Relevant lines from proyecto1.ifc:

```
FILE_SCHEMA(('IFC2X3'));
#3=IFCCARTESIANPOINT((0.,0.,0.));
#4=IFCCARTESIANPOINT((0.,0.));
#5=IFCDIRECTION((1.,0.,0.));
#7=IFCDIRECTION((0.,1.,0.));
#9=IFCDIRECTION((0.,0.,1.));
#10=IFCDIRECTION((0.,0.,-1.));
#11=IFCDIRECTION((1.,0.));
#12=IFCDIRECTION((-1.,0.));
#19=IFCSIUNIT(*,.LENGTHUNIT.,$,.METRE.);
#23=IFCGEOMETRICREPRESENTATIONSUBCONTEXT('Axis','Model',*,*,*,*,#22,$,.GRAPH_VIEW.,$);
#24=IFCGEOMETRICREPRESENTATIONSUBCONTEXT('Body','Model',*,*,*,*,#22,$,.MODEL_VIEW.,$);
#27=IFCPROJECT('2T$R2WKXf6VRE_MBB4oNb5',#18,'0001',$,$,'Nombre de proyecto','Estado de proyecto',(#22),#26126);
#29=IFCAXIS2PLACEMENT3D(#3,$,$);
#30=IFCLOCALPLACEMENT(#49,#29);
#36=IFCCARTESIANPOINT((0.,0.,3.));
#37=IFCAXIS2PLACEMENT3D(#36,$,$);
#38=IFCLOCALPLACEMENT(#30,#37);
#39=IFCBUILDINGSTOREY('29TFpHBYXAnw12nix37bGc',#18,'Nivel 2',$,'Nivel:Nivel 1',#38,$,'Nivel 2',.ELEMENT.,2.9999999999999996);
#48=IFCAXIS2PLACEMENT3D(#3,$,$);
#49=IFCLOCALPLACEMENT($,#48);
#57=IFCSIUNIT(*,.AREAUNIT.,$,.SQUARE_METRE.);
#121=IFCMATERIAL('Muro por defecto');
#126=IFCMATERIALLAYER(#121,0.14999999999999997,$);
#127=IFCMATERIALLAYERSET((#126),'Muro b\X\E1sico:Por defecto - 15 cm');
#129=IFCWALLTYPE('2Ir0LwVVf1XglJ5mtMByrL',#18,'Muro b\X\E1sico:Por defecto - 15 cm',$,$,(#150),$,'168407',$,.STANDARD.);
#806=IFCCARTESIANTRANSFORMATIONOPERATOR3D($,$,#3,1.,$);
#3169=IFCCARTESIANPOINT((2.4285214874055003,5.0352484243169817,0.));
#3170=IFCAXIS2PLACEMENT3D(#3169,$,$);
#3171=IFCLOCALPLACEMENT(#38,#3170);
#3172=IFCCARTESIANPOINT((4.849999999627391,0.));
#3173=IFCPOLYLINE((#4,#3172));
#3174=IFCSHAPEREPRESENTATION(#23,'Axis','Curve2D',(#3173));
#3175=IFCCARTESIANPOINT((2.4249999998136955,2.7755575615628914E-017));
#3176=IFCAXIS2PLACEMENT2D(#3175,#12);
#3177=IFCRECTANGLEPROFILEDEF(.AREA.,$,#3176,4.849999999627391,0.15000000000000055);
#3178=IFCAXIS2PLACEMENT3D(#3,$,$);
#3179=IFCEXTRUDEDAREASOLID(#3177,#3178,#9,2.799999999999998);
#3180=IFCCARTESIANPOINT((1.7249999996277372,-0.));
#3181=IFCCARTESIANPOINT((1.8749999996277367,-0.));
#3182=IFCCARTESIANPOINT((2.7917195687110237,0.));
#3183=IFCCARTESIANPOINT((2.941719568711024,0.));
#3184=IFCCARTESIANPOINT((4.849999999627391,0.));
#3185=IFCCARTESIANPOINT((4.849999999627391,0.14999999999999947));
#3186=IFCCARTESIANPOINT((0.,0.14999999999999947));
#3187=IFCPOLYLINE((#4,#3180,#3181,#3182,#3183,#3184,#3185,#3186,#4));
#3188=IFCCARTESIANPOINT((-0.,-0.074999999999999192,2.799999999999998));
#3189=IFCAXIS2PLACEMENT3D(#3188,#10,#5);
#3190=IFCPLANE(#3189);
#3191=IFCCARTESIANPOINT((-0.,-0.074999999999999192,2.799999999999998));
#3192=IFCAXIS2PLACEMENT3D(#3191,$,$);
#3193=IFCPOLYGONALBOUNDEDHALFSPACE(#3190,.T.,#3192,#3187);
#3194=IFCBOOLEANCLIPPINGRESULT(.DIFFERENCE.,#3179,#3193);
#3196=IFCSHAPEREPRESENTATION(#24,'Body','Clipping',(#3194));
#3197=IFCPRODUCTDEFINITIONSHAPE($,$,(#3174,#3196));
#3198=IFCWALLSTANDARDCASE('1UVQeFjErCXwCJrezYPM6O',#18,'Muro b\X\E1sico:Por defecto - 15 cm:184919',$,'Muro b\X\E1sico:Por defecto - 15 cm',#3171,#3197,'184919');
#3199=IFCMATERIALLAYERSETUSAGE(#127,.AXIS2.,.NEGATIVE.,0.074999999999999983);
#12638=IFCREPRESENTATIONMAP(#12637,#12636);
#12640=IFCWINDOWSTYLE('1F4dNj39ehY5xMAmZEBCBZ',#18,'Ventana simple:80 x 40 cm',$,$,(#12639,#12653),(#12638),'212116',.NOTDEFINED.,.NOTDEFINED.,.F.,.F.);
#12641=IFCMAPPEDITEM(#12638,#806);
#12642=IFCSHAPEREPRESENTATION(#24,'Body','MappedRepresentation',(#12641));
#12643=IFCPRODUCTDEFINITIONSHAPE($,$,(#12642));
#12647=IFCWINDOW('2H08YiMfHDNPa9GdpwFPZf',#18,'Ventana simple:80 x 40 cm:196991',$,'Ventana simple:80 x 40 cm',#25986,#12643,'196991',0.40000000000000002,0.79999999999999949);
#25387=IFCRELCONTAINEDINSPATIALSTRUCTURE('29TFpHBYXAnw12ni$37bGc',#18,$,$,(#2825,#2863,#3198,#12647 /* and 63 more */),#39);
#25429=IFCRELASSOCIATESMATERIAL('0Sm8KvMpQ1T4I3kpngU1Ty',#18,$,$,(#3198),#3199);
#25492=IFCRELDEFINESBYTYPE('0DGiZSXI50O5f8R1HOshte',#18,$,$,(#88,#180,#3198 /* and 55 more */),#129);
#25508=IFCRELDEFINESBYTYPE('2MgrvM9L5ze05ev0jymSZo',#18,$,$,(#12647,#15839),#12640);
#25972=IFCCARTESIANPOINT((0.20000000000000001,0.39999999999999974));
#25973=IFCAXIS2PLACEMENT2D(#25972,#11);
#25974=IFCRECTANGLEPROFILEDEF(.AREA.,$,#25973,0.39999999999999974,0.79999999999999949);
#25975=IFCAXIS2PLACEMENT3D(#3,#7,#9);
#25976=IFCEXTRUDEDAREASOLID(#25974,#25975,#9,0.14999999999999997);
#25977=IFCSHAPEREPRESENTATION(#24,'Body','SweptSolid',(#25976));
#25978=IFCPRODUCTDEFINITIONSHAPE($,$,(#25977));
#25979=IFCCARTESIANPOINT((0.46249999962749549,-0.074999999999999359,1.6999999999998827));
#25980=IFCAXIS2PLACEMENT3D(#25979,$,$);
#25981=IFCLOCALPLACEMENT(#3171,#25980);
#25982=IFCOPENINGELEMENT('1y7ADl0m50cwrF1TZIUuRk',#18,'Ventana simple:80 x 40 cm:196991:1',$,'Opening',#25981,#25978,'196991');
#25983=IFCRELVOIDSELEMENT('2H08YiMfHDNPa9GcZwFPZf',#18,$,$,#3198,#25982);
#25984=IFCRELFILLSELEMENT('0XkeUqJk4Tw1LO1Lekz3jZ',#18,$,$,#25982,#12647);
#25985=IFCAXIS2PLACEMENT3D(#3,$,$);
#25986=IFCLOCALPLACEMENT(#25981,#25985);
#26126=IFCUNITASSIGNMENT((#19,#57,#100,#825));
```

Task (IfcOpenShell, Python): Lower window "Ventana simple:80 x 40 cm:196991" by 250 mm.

```python
import numpy as np
import ifcopenshell
import ifcopenshell.api.geometry
import ifcopenshell.util.placement
import ifcopenshell.util.unit

model = ifcopenshell.open("proyecto1.ifc")
unit_scale = ifcopenshell.util.unit.calculate_unit_scale(model)

window = model.by_guid("2H08YiMfHDNPa9GdpwFPZf")
opening = window.FillsVoids[0].RelatingOpeningElement
dz = -0.25

shift = np.array([0.0, 0.0, dz])
# The window is placed relative to its opening, so it follows when the opening moves.
matrix = ifcopenshell.util.placement.get_local_placement(opening.ObjectPlacement)
matrix[:3, 3] += shift
ifcopenshell.api.geometry.edit_object_placement(
    model, product=opening, matrix=matrix, is_si=False, should_transform_children=True
)

print(f"moved by {dz * unit_scale:+.3f} m")

model.write("proyecto1_edited.ifc")
```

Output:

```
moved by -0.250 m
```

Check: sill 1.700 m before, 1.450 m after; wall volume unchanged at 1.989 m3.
